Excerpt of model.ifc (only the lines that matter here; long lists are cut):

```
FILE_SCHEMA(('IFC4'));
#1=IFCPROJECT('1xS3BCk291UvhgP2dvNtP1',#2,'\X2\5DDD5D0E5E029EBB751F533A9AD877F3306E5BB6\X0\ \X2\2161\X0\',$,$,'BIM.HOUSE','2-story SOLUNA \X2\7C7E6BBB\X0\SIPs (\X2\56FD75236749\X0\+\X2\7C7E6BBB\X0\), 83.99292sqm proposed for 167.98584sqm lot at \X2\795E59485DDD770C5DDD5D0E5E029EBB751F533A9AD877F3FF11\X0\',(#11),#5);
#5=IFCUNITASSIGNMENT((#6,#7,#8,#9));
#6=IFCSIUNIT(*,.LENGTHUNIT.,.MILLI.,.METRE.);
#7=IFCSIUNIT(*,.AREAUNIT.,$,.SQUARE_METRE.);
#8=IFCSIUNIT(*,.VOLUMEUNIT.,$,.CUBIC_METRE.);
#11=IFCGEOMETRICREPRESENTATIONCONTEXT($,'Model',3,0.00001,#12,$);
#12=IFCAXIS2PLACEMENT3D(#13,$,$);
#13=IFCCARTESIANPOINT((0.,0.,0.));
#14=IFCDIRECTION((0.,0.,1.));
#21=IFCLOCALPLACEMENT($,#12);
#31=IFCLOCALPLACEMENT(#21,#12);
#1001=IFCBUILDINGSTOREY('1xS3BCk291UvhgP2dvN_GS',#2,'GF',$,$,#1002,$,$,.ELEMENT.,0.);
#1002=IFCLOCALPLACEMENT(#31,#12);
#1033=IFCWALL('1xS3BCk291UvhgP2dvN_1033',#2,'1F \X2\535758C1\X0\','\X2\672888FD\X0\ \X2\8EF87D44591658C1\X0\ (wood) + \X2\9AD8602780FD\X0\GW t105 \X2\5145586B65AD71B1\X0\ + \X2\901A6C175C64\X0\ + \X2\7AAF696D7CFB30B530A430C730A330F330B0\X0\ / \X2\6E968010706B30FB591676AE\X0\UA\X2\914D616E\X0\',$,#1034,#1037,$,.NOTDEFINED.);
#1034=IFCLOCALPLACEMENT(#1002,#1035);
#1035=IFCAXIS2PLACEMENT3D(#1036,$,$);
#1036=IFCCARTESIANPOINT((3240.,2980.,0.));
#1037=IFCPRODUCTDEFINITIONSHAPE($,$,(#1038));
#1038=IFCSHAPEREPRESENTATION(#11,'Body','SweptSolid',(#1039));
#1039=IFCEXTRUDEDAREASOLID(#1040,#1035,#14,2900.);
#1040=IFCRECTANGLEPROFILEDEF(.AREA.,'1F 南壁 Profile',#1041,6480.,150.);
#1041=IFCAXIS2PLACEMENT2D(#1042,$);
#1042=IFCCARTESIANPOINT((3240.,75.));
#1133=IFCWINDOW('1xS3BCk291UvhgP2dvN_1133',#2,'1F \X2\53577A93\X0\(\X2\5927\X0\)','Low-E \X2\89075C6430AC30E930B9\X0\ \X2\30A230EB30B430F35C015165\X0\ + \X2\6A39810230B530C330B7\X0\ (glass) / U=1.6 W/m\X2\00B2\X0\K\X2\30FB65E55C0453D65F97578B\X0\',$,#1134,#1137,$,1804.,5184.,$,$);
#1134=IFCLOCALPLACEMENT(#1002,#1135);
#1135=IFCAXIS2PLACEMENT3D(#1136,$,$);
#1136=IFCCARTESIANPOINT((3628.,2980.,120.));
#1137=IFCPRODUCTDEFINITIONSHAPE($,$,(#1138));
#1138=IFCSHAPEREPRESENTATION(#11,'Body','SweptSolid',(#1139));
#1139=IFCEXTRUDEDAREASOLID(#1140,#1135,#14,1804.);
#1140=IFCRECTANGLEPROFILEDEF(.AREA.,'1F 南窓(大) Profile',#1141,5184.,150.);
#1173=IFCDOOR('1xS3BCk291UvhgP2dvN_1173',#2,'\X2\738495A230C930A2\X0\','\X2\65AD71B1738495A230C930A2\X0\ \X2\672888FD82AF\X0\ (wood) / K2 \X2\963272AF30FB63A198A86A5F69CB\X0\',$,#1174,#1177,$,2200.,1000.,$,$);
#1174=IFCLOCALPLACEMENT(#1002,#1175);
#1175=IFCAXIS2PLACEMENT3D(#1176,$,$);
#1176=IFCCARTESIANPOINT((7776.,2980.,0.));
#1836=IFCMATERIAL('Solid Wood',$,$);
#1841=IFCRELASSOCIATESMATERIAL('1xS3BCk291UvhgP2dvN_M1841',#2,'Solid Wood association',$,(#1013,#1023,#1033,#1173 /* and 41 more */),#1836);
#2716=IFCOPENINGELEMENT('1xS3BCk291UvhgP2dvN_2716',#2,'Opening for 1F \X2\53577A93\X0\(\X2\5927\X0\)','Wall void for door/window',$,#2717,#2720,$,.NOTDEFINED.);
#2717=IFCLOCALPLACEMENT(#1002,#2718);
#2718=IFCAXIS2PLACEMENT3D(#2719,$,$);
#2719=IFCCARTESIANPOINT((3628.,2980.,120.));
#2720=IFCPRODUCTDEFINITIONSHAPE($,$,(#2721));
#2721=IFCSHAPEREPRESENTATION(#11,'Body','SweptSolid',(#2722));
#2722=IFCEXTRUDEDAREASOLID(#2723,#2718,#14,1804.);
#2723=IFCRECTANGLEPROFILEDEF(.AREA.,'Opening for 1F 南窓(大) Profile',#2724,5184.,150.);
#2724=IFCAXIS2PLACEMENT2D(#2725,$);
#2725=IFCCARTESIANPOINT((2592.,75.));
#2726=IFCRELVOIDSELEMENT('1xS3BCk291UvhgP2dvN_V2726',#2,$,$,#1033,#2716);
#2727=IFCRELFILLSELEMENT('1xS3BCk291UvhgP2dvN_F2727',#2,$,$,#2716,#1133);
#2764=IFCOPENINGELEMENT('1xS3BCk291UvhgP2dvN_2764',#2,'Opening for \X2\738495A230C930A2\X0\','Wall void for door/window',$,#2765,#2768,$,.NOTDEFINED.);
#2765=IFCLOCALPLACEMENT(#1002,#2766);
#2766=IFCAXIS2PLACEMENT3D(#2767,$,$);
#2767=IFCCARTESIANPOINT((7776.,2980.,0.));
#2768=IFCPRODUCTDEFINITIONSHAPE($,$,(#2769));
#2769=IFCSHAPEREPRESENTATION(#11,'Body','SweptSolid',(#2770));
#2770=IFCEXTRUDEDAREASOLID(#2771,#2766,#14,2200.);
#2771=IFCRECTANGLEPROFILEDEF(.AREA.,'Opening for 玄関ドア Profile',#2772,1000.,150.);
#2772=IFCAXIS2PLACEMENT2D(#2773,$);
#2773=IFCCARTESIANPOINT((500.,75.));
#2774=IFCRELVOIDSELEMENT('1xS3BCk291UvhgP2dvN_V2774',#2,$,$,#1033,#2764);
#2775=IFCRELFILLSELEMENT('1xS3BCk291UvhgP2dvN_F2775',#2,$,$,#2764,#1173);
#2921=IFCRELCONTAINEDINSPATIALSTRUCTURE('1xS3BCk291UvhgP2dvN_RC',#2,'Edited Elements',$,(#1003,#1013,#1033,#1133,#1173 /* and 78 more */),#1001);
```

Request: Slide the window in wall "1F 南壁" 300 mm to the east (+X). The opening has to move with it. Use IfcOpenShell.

```python
import ifcopenshell
import ifcopenshell.api.geometry
import ifcopenshell.util.placement

model = ifcopenshell.open("model.ifc")

window = model.by_guid("1xS3BCk291UvhgP2dvN_1133")
opening = window.FillsVoids[0].RelatingOpeningElement
wall = opening.VoidsElements[0].RelatingBuildingElement

wall_matrix = ifcopenshell.util.placement.get_local_placement(wall.ObjectPlacement)
shift = wall_matrix[:3, 0] * 300.0
before = ifcopenshell.util.placement.get_local_placement(window.ObjectPlacement)[:3, 3].copy()

# The window is not placed relative to its opening, so move both.
for product in (opening, window):
    matrix = ifcopenshell.util.placement.get_local_placement(product.ObjectPlacement)
    matrix[:3, 3] += shift
    ifcopenshell.api.geometry.edit_object_placement(model, product=product, matrix=matrix, is_si=False)

after = ifcopenshell.util.placement.get_local_placement(window.ObjectPlacement)[:3, 3]
print("window moved by", (after - before).round(3) + 0.0)

model.write("model_edited.ifc")
```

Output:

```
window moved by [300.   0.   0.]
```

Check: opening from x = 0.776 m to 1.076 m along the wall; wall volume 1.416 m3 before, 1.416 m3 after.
